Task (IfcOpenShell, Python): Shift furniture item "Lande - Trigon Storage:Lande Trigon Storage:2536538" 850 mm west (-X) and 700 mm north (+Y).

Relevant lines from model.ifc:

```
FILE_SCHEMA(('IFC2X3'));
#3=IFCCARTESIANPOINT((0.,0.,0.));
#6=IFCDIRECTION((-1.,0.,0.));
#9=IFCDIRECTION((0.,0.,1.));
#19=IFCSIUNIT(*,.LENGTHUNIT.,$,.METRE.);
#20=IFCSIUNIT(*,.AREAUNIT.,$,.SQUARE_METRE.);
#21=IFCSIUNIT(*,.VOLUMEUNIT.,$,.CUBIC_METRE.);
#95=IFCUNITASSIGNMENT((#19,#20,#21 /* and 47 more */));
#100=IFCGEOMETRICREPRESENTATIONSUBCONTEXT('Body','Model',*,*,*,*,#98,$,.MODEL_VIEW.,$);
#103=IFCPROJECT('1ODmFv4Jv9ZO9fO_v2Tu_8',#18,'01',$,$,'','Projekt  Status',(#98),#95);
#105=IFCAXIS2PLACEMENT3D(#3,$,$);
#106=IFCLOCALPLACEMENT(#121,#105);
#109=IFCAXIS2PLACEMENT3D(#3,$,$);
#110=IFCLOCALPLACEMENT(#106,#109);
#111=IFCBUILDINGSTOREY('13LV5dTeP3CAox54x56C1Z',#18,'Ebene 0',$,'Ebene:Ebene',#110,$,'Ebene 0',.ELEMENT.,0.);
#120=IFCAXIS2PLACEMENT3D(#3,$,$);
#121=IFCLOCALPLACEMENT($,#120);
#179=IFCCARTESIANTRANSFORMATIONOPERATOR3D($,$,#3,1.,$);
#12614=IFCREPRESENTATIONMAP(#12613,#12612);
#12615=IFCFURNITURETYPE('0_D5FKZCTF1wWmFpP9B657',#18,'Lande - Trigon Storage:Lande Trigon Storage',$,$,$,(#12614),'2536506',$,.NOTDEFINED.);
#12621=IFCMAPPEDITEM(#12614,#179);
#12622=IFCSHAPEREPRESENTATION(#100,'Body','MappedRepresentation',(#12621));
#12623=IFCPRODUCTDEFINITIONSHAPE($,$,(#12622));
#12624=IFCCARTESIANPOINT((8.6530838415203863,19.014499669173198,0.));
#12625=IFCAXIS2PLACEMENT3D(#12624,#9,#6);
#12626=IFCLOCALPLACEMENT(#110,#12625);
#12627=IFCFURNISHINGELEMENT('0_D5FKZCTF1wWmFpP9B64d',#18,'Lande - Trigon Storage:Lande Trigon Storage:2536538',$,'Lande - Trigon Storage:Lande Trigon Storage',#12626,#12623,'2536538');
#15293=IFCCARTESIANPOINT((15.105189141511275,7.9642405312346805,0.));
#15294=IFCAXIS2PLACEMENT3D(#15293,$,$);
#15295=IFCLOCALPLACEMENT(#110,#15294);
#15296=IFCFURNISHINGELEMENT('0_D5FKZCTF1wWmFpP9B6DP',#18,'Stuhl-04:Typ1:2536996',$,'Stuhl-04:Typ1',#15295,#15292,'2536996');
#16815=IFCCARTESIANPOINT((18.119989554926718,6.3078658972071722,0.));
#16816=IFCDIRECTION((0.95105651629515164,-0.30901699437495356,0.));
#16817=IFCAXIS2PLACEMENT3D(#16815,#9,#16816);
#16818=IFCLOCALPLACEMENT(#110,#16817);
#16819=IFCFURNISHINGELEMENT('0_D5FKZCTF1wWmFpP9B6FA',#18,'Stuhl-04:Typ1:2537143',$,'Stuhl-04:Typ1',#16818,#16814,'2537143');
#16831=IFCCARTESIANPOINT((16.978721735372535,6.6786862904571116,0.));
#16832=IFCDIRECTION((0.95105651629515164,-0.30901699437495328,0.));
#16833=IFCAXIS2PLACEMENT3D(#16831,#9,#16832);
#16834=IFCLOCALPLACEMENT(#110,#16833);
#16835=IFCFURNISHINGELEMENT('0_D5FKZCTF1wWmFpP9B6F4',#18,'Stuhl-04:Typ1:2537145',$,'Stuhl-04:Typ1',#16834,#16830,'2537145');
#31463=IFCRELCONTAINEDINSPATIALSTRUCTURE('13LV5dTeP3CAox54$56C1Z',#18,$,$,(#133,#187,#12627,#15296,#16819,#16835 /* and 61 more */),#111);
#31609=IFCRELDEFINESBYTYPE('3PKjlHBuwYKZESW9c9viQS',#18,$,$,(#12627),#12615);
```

```python
import ifcopenshell
import ifcopenshell.api.geometry
import ifcopenshell.util.placement
import ifcopenshell.util.unit

model = ifcopenshell.open("model.ifc")
unit_scale = ifcopenshell.util.unit.calculate_unit_scale(model)

item = model.by_guid("0_D5FKZCTF1wWmFpP9B64d")
matrix = ifcopenshell.util.placement.get_local_placement(item.ObjectPlacement)
matrix[0, 3] -= 0.85 / unit_scale
matrix[1, 3] += 0.7 / unit_scale
ifcopenshell.api.geometry.edit_object_placement(model, product=item, matrix=matrix, is_si=False)

print(ifcopenshell.util.placement.get_local_placement(item.ObjectPlacement).round(3) + 0.0)

model.write("model-out.ifc")
```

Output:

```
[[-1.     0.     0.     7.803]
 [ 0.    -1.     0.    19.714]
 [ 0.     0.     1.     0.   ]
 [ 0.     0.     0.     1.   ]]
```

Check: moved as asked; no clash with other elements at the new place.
